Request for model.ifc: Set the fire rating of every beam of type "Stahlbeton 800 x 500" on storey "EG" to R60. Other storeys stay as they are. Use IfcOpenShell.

First a look at what the model holds.

```python
import ifcopenshell
import ifcopenshell.util.element

model = ifcopenshell.open("model.ifc")
print(model.schema)
storey = next(s for s in model.by_type("IfcBuildingStorey") if s.Name == "EG")
beams = [e for e in ifcopenshell.util.element.get_decomposition(storey) if e.is_a("IfcBeam")]
seen = {}
for e in beams:
    element_type = ifcopenshell.util.element.get_type(e)
    key = (element_type.Name if element_type != e and element_type else None, ifcopenshell.util.element.get_pset(e, "Pset_BeamCommon", "FireRating"))
    seen[key] = seen.get(key, 0) + 1
for (name, value), count in sorted(seen.items(), key=str):
    print(count, "x", name, "|", value)
```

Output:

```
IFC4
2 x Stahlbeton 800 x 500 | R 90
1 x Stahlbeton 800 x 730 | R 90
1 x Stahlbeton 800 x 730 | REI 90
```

```python
import ifcopenshell
import ifcopenshell.api.pset
import ifcopenshell.util.element

model = ifcopenshell.open("model.ifc")

storey = next(s for s in model.by_type("IfcBuildingStorey") if s.Name == "EG")
beams = [e for e in ifcopenshell.util.element.get_decomposition(storey) if e.is_a("IfcBeam")]

count = 0
for e in beams:
    element_type = ifcopenshell.util.element.get_type(e)
    if element_type in (None, e) or element_type.Name != "Stahlbeton 800 x 500":
        continue
    # add_pset returns the element's existing set when there is one.
    pset = ifcopenshell.api.pset.add_pset(model, product=e, name="Pset_BeamCommon")
    ifcopenshell.api.pset.edit_pset(model, pset=pset, properties={"FireRating": "R60"})
    count += 1

print(count, "beams updated")

model.write("model_updated.ifc")
```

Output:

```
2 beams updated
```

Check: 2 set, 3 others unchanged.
